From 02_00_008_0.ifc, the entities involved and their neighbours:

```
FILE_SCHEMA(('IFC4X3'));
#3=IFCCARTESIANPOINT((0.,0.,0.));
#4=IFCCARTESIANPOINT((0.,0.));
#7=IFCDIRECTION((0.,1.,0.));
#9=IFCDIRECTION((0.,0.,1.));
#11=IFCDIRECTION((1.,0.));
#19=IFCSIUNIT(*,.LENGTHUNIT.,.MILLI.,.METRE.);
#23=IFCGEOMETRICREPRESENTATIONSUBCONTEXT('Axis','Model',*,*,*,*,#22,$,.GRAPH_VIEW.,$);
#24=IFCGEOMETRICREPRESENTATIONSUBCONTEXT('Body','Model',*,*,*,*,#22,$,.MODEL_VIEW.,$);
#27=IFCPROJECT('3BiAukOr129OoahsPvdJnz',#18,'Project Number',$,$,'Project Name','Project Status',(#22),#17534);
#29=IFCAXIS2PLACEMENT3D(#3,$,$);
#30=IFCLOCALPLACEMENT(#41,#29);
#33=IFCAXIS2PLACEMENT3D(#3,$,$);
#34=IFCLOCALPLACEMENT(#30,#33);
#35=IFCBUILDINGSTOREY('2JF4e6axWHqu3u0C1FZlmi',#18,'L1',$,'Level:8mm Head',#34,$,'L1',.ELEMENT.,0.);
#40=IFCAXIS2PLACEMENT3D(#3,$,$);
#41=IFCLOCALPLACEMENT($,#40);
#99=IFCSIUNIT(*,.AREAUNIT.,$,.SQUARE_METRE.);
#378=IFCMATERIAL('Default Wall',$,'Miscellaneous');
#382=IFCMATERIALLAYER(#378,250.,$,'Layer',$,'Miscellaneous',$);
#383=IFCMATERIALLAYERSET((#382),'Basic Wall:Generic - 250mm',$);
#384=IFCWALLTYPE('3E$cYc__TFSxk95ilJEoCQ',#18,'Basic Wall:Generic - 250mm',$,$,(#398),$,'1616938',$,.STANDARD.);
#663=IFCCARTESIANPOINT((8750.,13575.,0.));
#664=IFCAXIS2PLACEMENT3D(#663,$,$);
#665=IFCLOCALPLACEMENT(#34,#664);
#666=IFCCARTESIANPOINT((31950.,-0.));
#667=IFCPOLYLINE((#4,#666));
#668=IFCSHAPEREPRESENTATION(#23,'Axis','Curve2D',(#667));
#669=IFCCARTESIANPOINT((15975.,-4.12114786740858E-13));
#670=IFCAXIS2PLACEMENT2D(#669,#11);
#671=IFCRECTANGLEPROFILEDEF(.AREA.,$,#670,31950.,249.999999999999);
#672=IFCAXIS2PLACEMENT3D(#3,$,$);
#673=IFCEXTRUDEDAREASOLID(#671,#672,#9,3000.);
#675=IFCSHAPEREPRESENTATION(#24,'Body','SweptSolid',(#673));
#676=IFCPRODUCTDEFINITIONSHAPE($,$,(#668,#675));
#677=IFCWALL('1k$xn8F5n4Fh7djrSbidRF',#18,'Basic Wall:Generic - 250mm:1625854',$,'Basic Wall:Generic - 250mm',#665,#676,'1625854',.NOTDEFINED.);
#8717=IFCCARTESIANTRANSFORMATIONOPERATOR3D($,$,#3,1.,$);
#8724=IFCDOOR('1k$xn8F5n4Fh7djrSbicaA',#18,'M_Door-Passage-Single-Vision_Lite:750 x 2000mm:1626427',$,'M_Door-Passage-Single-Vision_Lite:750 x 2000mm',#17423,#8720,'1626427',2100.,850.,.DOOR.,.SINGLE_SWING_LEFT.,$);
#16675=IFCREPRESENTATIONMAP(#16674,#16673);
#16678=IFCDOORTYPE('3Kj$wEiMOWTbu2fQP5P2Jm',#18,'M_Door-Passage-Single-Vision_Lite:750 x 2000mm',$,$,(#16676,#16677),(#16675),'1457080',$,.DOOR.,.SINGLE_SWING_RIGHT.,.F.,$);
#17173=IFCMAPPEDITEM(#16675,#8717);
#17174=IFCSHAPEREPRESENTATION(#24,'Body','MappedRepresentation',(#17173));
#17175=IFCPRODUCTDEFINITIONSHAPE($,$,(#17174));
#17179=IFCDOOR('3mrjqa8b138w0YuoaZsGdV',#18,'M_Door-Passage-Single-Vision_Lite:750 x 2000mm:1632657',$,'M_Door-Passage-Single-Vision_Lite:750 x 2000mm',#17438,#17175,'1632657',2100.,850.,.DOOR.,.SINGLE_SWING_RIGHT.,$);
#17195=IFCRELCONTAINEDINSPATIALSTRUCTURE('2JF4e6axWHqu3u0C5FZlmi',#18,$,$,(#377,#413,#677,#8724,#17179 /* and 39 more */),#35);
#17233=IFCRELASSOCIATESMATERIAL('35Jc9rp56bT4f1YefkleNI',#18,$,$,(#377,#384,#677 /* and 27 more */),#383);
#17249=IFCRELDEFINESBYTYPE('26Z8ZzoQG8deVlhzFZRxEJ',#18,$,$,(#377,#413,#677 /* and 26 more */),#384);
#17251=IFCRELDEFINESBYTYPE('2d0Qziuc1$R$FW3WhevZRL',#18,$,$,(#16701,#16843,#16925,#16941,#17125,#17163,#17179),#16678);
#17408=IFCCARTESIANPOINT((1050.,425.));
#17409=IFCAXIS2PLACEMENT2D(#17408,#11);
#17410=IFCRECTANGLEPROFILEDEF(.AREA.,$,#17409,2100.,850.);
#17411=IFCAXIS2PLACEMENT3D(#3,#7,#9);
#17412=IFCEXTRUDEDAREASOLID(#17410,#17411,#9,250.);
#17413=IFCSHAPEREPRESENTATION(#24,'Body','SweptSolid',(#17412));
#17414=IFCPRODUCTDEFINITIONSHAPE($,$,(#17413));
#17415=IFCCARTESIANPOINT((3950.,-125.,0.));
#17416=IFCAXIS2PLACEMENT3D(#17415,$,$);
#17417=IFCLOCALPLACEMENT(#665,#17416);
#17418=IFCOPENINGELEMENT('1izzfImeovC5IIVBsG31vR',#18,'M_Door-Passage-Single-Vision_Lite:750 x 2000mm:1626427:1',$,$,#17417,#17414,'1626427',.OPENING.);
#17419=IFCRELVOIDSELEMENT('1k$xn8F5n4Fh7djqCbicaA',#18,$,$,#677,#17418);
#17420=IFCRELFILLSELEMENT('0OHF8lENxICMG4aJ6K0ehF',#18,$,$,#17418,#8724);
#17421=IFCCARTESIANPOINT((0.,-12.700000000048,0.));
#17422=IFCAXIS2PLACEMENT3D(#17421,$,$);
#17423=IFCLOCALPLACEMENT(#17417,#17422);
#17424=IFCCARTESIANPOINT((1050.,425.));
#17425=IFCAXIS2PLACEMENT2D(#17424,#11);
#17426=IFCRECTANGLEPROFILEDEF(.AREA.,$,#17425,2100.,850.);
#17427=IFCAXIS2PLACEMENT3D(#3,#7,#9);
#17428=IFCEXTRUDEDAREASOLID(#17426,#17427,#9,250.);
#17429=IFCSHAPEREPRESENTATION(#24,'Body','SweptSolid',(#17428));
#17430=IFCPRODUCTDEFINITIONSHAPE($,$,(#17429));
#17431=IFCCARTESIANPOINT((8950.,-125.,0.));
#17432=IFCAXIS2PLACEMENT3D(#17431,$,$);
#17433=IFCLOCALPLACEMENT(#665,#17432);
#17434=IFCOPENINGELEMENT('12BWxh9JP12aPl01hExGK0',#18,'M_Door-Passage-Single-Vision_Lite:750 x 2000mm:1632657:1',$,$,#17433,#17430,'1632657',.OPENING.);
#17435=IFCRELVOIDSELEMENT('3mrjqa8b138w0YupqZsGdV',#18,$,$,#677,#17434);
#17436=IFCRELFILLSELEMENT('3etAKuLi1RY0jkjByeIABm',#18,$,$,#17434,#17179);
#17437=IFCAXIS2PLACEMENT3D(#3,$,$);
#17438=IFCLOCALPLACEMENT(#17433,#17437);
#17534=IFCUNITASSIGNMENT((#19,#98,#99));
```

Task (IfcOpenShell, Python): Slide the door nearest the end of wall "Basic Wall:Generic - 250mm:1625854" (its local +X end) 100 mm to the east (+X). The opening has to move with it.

```python
import ifcopenshell
import ifcopenshell.api.geometry
import ifcopenshell.util.placement
import ifcopenshell.util.unit

model = ifcopenshell.open("02_00_008_0.ifc")
unit_scale = ifcopenshell.util.unit.calculate_unit_scale(model)

door = model.by_id(17179)
opening = door.FillsVoids[0].RelatingOpeningElement
wall = opening.VoidsElements[0].RelatingBuildingElement

wall_matrix = ifcopenshell.util.placement.get_local_placement(wall.ObjectPlacement)
shift = wall_matrix[:3, 0] * 0.1 / unit_scale
before = ifcopenshell.util.placement.get_local_placement(door.ObjectPlacement)[:3, 3].copy()

# The door is placed relative to its opening, so it follows when the opening moves.
matrix = ifcopenshell.util.placement.get_local_placement(opening.ObjectPlacement)
matrix[:3, 3] += shift
ifcopenshell.api.geometry.edit_object_placement(
    model, product=opening, matrix=matrix, is_si=False, should_transform_children=True
)

after = ifcopenshell.util.placement.get_local_placement(door.ObjectPlacement)[:3, 3]
print("door moved by", (after - before).round(3) + 0.0)

model.write("02_00_008_0_v2.ifc")
```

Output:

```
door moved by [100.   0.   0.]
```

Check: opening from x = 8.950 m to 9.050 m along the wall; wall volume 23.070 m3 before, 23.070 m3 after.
